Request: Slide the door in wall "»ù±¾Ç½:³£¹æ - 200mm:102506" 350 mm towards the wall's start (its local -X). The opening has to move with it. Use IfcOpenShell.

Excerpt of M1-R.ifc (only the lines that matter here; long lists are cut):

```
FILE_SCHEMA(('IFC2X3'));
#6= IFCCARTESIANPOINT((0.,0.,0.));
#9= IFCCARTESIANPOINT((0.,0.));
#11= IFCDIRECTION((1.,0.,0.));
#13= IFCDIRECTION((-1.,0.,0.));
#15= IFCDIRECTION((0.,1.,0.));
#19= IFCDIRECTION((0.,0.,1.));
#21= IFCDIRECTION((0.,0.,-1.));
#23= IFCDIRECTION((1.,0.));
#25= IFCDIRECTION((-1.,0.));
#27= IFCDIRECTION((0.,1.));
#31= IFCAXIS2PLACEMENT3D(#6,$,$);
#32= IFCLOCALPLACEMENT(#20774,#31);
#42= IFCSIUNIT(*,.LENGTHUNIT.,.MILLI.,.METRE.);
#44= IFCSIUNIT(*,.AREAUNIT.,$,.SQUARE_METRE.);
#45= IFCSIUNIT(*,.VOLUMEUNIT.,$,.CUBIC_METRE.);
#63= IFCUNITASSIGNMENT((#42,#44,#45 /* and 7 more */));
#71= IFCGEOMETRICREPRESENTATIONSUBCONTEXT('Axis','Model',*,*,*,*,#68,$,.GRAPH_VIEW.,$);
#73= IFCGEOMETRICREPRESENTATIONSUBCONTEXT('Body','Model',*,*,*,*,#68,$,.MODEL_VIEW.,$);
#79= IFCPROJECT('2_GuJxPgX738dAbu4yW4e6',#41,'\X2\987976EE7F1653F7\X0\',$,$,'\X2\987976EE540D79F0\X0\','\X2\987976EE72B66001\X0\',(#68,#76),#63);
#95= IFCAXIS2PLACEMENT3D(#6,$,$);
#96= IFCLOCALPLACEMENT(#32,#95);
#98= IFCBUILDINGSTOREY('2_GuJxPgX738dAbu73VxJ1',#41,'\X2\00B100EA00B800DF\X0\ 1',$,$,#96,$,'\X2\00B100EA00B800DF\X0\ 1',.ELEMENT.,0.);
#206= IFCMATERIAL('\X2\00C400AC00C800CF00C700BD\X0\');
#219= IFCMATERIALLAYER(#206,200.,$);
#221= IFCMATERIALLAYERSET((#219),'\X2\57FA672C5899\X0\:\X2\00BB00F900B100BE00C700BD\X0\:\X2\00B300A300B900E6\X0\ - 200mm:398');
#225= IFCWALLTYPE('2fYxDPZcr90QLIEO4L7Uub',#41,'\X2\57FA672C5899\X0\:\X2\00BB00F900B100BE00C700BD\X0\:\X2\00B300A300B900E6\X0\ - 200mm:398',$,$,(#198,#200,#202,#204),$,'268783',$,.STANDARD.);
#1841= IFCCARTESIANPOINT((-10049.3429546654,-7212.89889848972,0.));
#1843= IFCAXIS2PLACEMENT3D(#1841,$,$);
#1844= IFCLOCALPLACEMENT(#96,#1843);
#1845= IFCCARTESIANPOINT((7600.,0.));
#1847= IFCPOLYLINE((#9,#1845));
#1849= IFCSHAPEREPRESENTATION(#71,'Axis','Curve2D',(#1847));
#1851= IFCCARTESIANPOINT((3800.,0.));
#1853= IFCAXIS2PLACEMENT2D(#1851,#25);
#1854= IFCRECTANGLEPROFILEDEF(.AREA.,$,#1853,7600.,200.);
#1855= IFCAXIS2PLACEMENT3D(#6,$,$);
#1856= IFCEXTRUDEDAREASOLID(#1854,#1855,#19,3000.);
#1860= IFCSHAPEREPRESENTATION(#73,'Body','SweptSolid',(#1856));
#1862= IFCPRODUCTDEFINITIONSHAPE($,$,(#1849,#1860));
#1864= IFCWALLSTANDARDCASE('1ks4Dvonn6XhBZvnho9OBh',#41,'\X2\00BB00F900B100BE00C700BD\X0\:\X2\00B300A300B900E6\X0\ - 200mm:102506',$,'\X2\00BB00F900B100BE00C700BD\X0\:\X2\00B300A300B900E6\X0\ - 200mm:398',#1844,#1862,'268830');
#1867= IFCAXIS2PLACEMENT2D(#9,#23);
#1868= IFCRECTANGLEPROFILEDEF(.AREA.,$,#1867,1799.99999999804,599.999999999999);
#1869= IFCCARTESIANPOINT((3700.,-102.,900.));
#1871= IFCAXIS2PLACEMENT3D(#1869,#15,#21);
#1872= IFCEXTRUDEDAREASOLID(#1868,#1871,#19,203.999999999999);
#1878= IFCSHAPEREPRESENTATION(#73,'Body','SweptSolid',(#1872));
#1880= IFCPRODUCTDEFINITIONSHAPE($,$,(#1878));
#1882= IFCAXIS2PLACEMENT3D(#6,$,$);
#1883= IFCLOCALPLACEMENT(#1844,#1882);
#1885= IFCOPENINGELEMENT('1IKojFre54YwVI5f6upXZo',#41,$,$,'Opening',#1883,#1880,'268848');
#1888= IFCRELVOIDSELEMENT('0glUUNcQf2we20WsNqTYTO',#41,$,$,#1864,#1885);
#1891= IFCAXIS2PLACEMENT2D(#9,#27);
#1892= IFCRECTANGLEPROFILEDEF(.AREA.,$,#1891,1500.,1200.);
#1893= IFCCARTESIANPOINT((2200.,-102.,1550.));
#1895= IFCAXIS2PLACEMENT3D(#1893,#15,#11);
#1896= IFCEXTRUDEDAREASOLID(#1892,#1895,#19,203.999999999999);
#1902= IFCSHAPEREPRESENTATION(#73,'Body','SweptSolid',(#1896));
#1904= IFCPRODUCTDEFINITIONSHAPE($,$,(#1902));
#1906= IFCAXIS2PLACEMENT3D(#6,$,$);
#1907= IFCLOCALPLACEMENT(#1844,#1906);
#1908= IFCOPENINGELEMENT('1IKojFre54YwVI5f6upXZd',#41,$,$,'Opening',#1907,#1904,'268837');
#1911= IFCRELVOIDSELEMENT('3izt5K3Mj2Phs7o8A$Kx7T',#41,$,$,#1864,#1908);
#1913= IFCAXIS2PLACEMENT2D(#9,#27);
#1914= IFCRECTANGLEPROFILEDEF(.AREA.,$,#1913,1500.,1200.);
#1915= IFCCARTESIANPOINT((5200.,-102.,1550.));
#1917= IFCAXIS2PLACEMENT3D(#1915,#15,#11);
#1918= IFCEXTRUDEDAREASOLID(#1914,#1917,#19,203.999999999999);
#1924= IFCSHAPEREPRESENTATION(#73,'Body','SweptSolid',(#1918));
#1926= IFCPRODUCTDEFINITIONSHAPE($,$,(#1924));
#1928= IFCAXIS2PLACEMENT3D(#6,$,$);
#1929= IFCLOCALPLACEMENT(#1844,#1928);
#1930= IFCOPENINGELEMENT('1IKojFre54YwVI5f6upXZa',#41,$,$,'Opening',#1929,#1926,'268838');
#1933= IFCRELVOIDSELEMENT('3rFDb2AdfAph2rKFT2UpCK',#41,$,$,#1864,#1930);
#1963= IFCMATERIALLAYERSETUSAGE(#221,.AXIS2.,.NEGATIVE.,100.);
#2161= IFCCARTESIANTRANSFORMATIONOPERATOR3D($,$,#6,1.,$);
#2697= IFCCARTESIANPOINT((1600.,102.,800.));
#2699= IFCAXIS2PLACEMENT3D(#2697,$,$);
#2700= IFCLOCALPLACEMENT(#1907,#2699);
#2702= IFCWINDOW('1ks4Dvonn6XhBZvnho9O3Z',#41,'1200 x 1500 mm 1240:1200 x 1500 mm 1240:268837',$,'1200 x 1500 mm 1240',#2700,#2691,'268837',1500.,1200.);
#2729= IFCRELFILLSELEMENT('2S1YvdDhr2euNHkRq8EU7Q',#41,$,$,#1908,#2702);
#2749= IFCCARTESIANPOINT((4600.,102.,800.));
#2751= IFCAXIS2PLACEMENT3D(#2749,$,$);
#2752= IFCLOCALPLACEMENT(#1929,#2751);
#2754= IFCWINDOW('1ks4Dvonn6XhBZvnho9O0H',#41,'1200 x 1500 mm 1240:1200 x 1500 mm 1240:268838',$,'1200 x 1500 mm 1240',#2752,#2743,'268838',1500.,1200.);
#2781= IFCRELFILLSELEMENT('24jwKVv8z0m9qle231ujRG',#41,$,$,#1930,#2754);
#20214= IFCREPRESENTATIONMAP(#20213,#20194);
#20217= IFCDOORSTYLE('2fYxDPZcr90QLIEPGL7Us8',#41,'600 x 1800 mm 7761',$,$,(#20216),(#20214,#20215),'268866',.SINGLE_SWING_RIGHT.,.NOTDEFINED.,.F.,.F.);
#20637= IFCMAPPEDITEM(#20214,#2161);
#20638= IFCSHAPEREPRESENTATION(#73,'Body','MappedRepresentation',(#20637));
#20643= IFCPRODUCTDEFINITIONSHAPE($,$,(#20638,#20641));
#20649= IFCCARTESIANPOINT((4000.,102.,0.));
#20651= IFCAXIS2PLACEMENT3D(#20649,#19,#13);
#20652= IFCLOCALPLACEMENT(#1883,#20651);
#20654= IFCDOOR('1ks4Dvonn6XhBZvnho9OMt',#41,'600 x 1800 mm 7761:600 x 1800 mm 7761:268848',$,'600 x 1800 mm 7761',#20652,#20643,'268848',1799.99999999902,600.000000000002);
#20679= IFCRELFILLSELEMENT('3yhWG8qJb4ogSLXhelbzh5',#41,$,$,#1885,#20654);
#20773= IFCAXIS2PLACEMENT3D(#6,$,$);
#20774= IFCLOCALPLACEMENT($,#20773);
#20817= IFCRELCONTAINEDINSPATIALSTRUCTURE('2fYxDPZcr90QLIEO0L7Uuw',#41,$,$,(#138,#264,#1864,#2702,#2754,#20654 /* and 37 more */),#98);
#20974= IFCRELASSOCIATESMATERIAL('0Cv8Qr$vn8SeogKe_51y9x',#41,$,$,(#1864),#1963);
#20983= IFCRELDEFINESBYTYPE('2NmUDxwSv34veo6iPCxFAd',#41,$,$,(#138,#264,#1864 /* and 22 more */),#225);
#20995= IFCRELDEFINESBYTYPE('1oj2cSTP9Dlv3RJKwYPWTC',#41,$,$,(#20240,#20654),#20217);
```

```python
import ifcopenshell
import ifcopenshell.api.geometry
import ifcopenshell.util.placement

model = ifcopenshell.open("M1-R.ifc")

door = model.by_guid("1ks4Dvonn6XhBZvnho9OMt")
opening = door.FillsVoids[0].RelatingOpeningElement
wall = opening.VoidsElements[0].RelatingBuildingElement

wall_matrix = ifcopenshell.util.placement.get_local_placement(wall.ObjectPlacement)
shift = wall_matrix[:3, 0] * -350.0
before = ifcopenshell.util.placement.get_local_placement(door.ObjectPlacement)[:3, 3].copy()

# The door is placed relative to its opening, so it follows when the opening moves.
matrix = ifcopenshell.util.placement.get_local_placement(opening.ObjectPlacement)
matrix[:3, 3] += shift
ifcopenshell.api.geometry.edit_object_placement(
    model, product=opening, matrix=matrix, is_si=False, should_transform_children=True
)

after = ifcopenshell.util.placement.get_local_placement(door.ObjectPlacement)[:3, 3]
print("door moved by", (after - before).round(3) + 0.0)

model.write("M1-R_edited.ifc")
```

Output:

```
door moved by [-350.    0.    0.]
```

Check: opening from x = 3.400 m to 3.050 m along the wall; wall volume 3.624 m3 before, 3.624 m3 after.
